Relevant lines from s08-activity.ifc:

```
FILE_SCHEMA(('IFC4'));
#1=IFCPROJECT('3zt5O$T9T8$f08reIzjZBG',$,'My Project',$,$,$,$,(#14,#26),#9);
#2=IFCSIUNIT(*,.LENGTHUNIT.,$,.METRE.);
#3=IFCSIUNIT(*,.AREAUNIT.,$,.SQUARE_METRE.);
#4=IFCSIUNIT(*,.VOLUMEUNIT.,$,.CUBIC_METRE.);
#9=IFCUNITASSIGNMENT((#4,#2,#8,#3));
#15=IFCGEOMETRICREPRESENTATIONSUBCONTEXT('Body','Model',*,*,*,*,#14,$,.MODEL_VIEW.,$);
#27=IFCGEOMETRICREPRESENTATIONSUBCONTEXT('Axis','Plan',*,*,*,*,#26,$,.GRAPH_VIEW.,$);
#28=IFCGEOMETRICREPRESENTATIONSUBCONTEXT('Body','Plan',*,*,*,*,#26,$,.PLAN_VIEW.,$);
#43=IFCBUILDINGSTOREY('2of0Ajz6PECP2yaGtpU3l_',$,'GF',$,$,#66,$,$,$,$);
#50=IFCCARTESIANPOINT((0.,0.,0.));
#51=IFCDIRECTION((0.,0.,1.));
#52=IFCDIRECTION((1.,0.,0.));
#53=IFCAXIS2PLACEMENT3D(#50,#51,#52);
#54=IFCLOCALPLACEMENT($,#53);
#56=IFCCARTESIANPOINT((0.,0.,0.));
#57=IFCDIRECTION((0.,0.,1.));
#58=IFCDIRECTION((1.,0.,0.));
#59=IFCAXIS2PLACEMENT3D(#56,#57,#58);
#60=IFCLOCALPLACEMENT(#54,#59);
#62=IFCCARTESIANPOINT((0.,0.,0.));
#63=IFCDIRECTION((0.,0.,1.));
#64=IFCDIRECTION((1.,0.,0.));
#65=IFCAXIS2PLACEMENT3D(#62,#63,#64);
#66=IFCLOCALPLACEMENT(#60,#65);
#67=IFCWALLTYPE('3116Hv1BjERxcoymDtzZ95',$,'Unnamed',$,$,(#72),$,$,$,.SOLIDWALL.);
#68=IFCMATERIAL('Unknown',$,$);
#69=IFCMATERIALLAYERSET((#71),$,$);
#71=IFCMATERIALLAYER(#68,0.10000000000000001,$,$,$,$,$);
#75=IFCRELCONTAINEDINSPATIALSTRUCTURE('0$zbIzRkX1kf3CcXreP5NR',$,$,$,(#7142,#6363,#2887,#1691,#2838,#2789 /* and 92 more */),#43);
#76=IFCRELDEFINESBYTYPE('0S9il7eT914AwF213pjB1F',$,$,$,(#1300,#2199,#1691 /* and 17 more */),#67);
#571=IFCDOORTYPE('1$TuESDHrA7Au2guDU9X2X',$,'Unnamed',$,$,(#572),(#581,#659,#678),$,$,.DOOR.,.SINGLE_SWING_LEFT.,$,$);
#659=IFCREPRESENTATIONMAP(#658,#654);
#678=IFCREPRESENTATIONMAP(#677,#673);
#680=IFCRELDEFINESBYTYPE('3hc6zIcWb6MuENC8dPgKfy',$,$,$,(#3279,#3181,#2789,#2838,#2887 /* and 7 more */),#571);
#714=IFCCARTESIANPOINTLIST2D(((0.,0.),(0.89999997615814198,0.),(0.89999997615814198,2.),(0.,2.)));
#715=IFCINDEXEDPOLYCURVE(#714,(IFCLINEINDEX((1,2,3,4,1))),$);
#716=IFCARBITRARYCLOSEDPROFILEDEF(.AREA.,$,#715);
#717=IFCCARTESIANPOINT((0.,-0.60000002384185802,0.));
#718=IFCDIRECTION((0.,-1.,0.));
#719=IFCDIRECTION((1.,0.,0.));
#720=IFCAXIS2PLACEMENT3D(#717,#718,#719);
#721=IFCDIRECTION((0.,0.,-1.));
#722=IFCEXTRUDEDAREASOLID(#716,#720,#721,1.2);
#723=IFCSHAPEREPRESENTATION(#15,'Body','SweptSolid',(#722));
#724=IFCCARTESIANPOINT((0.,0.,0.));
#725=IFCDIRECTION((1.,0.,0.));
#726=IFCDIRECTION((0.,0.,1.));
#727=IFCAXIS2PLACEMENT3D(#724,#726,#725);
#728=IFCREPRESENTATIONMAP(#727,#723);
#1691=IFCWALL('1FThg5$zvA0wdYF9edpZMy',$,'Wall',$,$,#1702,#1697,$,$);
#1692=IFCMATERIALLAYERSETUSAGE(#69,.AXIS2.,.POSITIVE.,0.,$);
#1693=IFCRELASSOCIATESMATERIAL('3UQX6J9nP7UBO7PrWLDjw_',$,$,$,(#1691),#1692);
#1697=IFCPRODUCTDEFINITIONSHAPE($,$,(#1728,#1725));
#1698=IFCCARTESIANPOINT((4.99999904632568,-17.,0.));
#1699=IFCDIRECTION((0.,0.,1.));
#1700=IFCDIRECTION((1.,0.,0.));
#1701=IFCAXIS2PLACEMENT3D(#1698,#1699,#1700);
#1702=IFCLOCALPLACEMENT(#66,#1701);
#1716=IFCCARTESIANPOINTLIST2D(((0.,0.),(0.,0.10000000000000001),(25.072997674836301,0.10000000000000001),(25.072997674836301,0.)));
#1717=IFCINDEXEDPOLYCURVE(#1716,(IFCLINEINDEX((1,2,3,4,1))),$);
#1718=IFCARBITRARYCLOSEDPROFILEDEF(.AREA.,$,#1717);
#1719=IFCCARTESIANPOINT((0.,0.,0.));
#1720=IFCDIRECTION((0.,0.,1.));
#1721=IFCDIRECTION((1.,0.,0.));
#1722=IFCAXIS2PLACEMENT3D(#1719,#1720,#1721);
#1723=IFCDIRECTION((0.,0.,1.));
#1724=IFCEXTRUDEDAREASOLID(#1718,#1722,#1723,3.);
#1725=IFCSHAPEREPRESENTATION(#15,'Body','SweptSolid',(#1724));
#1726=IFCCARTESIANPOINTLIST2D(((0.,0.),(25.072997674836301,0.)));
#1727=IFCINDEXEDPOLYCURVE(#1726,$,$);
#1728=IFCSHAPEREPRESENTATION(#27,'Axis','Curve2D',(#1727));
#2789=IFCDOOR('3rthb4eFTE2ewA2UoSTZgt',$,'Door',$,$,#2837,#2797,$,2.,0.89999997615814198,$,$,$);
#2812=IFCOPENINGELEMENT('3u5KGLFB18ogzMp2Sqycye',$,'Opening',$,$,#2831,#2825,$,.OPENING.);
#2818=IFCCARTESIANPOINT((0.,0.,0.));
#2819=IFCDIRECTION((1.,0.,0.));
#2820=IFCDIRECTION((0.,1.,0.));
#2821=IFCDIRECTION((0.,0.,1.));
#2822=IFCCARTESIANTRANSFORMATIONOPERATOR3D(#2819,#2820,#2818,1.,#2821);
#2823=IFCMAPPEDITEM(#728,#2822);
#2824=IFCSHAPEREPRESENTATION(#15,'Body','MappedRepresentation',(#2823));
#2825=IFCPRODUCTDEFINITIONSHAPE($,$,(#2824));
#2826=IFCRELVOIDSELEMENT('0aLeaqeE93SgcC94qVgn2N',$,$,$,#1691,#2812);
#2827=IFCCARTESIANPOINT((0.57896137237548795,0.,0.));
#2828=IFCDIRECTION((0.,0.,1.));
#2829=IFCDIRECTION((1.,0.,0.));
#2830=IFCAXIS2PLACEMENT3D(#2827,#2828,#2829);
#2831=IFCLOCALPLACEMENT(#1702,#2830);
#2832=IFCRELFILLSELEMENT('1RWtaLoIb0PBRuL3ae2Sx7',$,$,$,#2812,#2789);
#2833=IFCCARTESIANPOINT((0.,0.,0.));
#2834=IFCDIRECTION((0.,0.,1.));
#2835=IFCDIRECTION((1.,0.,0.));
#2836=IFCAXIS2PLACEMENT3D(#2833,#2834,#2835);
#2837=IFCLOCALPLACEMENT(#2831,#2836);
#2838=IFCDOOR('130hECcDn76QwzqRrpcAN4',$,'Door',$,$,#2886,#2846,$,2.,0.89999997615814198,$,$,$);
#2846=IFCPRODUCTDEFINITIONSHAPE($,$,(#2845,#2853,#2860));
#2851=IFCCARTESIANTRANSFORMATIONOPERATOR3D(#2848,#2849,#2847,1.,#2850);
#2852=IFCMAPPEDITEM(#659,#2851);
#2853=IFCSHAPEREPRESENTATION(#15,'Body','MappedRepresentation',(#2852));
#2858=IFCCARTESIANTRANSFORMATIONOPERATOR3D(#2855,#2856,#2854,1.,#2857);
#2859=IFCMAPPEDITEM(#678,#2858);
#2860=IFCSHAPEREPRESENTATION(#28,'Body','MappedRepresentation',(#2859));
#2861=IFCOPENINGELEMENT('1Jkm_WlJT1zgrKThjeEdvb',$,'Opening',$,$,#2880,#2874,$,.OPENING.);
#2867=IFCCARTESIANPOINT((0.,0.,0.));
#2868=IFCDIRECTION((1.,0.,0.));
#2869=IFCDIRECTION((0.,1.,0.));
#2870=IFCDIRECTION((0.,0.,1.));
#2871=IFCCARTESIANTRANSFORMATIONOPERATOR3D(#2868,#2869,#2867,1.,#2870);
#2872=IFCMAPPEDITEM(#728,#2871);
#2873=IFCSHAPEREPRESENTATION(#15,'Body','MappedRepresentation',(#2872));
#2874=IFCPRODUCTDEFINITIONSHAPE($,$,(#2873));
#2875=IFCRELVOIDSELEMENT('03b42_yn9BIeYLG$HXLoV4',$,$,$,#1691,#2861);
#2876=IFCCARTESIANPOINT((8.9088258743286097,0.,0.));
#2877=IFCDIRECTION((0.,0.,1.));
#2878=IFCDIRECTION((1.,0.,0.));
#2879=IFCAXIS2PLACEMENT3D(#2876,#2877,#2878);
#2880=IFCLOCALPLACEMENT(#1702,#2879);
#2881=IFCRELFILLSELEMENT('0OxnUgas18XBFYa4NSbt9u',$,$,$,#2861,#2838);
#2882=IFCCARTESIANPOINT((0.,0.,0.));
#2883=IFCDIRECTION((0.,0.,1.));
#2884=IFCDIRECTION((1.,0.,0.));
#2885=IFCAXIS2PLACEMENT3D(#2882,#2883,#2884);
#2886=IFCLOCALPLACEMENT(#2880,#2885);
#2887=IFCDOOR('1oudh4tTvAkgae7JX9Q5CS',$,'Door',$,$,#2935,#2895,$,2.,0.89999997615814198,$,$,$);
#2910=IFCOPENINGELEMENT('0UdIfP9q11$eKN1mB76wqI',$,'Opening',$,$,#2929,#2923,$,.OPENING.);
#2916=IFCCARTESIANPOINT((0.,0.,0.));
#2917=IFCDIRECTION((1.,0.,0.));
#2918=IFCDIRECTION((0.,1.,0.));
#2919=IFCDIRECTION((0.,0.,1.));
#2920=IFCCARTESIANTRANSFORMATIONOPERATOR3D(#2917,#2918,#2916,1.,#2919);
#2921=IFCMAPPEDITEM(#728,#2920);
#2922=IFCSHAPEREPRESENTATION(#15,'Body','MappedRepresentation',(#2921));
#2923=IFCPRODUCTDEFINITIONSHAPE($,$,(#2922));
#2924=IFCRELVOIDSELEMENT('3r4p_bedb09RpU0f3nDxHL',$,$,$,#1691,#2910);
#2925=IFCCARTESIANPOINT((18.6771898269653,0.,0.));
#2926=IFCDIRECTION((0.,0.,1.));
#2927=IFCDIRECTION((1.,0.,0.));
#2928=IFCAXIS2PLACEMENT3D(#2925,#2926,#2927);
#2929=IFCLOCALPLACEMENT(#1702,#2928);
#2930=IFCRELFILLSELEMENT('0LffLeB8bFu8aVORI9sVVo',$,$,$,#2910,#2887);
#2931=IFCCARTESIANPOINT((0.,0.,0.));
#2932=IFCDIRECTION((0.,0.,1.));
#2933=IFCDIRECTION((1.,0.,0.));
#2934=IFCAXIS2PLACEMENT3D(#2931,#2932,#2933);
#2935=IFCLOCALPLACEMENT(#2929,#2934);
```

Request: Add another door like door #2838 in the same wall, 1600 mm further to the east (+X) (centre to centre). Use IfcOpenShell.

```python
import ifcopenshell
import ifcopenshell.api.feature
import ifcopenshell.api.geometry
import ifcopenshell.api.root
import ifcopenshell.geom
import ifcopenshell.util.element
import ifcopenshell.util.placement
import ifcopenshell.util.shape

model = ifcopenshell.open("s08-activity.ifc")
settings = ifcopenshell.geom.settings()


def volume(element):
    """Net volume in cubic metres, openings subtracted."""
    shape = ifcopenshell.geom.create_shape(settings, element)
    return ifcopenshell.util.shape.get_volume(shape.geometry)


door = model.by_guid("130hECcDn76QwzqRrpcAN4")
opening = door.FillsVoids[0].RelatingOpeningElement
wall = opening.VoidsElements[0].RelatingBuildingElement
before = volume(wall)
shift = ifcopenshell.util.placement.get_local_placement(wall.ObjectPlacement)[:3, 0] * 1.6

# copy_class copies the void relationship, type, container and properties, but no geometry.
new_opening = ifcopenshell.api.root.copy_class(model, product=opening)
new_opening.Representation = ifcopenshell.util.element.copy_deep(
    model, opening.Representation, exclude=["IfcGeometricRepresentationContext", "IfcRepresentationMap"]
)
new_door = ifcopenshell.api.root.copy_class(model, product=door)
new_door.Representation = ifcopenshell.util.element.copy_deep(
    model, door.Representation, exclude=["IfcGeometricRepresentationContext", "IfcRepresentationMap"]
)
ifcopenshell.api.feature.add_filling(model, opening=new_opening, element=new_door)

for old, new in ((opening, new_opening), (door, new_door)):
    matrix = ifcopenshell.util.placement.get_local_placement(old.ObjectPlacement)
    matrix[:3, 3] += shift
    ifcopenshell.api.geometry.edit_object_placement(model, product=new, matrix=matrix, is_si=False)

after = volume(wall)

print(f"wall volume {before:.3f} -> {after:.3f} m3")

model.write("s08-activity_edited.ifc")
```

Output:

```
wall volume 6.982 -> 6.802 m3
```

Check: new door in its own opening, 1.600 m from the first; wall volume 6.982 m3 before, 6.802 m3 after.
